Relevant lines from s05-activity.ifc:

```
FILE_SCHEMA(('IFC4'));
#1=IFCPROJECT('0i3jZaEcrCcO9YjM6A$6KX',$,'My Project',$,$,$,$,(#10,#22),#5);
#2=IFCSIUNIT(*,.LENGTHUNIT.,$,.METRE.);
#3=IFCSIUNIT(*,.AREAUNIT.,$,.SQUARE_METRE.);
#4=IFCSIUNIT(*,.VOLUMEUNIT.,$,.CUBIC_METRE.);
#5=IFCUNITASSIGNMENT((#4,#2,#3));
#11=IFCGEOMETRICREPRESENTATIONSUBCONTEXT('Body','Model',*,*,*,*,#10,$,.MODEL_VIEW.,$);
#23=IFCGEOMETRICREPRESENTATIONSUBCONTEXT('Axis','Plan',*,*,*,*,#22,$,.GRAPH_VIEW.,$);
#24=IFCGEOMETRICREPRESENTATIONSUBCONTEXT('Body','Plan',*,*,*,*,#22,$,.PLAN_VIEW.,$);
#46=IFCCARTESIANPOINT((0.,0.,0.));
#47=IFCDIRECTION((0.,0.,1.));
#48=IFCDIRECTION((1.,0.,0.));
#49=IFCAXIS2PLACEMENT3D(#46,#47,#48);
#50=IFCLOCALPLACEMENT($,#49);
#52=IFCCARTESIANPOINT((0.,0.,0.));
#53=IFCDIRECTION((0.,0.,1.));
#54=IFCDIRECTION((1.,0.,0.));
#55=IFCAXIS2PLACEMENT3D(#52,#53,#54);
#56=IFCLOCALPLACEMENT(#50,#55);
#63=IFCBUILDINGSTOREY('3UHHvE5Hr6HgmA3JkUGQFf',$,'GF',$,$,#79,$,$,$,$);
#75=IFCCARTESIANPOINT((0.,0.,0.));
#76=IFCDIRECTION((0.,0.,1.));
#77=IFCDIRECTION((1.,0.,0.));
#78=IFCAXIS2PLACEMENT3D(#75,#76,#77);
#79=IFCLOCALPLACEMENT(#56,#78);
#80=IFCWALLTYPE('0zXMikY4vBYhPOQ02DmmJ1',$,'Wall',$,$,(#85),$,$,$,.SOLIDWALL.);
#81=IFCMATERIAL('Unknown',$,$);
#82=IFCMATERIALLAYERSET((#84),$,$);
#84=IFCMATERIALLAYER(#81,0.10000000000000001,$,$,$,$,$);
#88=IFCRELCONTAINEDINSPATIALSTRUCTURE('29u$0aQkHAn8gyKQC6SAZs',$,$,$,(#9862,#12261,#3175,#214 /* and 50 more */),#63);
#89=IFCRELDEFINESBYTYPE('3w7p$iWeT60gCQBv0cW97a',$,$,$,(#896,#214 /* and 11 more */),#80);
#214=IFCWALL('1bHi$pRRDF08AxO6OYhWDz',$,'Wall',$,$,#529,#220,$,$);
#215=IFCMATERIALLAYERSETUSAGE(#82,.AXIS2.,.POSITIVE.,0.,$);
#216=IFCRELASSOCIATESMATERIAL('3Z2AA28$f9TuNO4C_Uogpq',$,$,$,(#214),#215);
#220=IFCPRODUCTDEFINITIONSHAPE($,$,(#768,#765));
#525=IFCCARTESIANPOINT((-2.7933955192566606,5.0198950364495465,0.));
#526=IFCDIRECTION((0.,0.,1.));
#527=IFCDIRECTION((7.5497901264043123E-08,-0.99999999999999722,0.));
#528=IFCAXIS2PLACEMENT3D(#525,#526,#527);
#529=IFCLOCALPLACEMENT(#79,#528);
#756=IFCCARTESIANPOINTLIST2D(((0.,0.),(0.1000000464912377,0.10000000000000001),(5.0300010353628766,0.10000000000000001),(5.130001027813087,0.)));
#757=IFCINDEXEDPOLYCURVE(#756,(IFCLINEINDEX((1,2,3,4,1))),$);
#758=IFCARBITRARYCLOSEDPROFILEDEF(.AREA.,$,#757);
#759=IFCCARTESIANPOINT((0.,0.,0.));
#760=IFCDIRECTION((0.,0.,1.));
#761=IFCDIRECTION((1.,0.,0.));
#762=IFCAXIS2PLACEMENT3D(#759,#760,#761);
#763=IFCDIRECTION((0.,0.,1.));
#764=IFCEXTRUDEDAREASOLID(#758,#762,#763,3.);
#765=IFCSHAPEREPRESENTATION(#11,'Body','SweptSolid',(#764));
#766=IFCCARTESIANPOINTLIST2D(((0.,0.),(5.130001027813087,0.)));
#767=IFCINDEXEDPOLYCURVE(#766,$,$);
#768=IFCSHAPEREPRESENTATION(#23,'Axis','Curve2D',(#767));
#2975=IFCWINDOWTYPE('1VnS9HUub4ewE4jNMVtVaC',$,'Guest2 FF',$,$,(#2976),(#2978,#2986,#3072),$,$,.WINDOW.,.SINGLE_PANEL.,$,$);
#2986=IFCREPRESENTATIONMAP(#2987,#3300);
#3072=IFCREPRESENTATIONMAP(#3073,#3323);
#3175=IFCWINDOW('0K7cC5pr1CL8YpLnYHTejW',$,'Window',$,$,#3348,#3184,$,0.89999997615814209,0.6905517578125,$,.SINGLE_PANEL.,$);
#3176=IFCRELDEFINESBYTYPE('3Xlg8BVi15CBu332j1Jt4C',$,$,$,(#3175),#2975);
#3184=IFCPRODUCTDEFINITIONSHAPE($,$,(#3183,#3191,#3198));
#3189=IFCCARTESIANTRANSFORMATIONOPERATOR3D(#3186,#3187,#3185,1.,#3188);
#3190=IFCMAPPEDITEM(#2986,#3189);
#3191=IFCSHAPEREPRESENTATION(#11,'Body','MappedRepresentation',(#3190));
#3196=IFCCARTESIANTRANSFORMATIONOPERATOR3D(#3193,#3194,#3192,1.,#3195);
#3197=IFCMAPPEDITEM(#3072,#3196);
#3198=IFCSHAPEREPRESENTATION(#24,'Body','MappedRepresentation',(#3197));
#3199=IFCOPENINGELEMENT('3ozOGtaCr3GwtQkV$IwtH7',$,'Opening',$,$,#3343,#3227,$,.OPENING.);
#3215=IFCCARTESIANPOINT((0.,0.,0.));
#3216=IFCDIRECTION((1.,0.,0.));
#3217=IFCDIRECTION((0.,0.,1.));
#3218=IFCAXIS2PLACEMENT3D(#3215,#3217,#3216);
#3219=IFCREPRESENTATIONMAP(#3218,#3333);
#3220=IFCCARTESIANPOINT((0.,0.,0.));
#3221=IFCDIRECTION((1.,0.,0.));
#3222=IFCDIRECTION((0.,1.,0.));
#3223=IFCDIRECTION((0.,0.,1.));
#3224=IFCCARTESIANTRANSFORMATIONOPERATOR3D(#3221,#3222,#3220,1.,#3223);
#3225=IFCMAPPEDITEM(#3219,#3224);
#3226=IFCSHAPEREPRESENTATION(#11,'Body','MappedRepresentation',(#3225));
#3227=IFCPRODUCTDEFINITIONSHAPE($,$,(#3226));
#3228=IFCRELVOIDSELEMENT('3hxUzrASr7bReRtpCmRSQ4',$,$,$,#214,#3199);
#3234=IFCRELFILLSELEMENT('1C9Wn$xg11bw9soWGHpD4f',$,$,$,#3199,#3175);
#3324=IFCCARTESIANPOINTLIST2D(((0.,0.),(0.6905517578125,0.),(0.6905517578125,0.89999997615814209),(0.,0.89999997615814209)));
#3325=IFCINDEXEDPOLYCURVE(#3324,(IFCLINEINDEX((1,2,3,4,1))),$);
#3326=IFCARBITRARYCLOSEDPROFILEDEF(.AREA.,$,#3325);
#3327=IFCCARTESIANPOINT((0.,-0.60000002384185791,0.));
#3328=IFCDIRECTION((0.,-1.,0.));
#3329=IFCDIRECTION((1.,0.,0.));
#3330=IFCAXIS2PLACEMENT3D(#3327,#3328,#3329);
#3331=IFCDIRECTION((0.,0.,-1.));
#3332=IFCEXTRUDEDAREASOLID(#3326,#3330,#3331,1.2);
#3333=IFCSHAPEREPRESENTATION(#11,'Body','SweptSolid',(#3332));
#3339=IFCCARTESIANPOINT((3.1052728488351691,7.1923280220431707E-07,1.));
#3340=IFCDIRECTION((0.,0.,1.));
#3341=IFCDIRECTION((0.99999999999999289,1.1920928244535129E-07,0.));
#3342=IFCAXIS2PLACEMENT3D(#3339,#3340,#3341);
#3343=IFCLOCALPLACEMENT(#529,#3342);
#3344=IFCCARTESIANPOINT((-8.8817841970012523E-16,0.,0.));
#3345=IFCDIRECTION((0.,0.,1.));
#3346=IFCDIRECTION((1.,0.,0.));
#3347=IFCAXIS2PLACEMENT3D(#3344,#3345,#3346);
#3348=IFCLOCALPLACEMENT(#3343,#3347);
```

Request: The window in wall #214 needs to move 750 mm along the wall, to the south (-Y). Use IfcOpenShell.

```python
import ifcopenshell
import ifcopenshell.api.geometry
import ifcopenshell.util.placement

model = ifcopenshell.open("s05-activity.ifc")

window = model.by_guid("0K7cC5pr1CL8YpLnYHTejW")
opening = window.FillsVoids[0].RelatingOpeningElement
wall = opening.VoidsElements[0].RelatingBuildingElement

wall_matrix = ifcopenshell.util.placement.get_local_placement(wall.ObjectPlacement)
shift = wall_matrix[:3, 0] * 0.75
before = ifcopenshell.util.placement.get_local_placement(window.ObjectPlacement)[:3, 3].copy()

# The window is placed relative to its opening, so it follows when the opening moves.
matrix = ifcopenshell.util.placement.get_local_placement(opening.ObjectPlacement)
matrix[:3, 3] += shift
ifcopenshell.api.geometry.edit_object_placement(
    model, product=opening, matrix=matrix, is_si=False, should_transform_children=True
)

after = ifcopenshell.util.placement.get_local_placement(window.ObjectPlacement)[:3, 3]
print("window moved by", (after - before).round(3) + 0.0)

model.write("s05-activity_edited.ifc")
```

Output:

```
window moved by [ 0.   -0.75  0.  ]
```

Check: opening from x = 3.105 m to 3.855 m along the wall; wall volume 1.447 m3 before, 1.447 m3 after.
